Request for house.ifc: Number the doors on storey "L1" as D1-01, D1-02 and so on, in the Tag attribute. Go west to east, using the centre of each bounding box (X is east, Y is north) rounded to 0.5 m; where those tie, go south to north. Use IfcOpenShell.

First a look at what the model holds.

```python
import ifcopenshell
import ifcopenshell.util.element
import ifcopenshell.util.placement

model = ifcopenshell.open("house.ifc")
print(model.schema)
storey = next(s for s in model.by_type("IfcBuildingStorey") if s.Name == "L1")
doors = [e for e in ifcopenshell.util.element.get_decomposition(storey) if e.is_a("IfcDoor")]
for e in sorted(doors, key=lambda e: e.id()):
    origin = ifcopenshell.util.placement.get_local_placement(e.ObjectPlacement)[:3, 3]
    print(e.id(), e.Tag, e.Name, origin.round(2) + 0.0, sep=" | ")
```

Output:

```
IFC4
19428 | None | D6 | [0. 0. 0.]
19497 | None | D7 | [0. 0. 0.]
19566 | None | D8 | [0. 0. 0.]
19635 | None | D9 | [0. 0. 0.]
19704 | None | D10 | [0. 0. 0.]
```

```python
import ifcopenshell
import ifcopenshell.geom
import ifcopenshell.util.element
import ifcopenshell.util.shape

model = ifcopenshell.open("house.ifc")
settings = ifcopenshell.geom.settings()
settings.set("use-world-coords", True)


def centre(element):
    shape = ifcopenshell.geom.create_shape(settings, element)
    return ifcopenshell.util.shape.get_bbox_centroid(shape.geometry)


storey = next(s for s in model.by_type("IfcBuildingStorey") if s.Name == "L1")
doors = [e for e in ifcopenshell.util.element.get_decomposition(storey) if e.is_a("IfcDoor")]

# Insertion points can sit at a corner or the storey origin, so sort by the geometry (in metres).
centres = {e: centre(e) for e in doors}
doors.sort(key=lambda e: (round(centres[e][0] / 0.5), centres[e][1]))

for i, e in enumerate(doors, start=1):
    number = f"D1-{i:02d}"
    e.Tag = number
    print(e.id(), number)

model.write("house_edited.ifc")
```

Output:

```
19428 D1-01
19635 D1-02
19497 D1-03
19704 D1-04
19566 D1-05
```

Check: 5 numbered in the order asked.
